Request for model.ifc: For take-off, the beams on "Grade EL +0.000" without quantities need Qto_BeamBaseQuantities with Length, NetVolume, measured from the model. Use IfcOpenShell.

First a look at what the model holds.

```python
import ifcopenshell
import ifcopenshell.util.element
import ifcopenshell.util.unit

model = ifcopenshell.open("model.ifc")
print(model.schema)
for unit_type in ("LENGTHUNIT", "AREAUNIT", "VOLUMEUNIT"):
    print(unit_type, ifcopenshell.util.unit.calculate_unit_scale(model, unit_type))
storey = next(s for s in model.by_type("IfcBuildingStorey") if s.Name == "Grade EL +0.000")
beams = [e for e in ifcopenshell.util.element.get_decomposition(storey) if e.is_a("IfcBeam")]
for e in sorted(beams, key=lambda e: e.id()):
    print(e.id(), e.is_a(), e.Name, list(ifcopenshell.util.element.get_psets(e, qtos_only=True)), sep=" | ")
```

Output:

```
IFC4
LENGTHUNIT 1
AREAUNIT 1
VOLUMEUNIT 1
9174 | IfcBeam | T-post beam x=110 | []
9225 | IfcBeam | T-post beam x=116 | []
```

```python
import ifcopenshell
import ifcopenshell.api.pset
import ifcopenshell.geom
import ifcopenshell.util.element
import ifcopenshell.util.shape
import ifcopenshell.util.unit

model = ifcopenshell.open("model.ifc")
unit_scale = ifcopenshell.util.unit.calculate_unit_scale(model)
volume_scale = ifcopenshell.util.unit.calculate_unit_scale(model, "VOLUMEUNIT")
settings = ifcopenshell.geom.settings()

storey = next(s for s in model.by_type("IfcBuildingStorey") if s.Name == "Grade EL +0.000")
beams = [e for e in ifcopenshell.util.element.get_decomposition(storey) if e.is_a("IfcBeam")]

for e in sorted(beams, key=lambda e: e.id()):
    if ifcopenshell.util.element.get_psets(e, qtos_only=True, should_inherit=False):
        continue
    # Geometry comes back in metres, in the element's own axes.
    shape = ifcopenshell.geom.create_shape(settings, e)
    values = {
        "Length": ifcopenshell.util.shape.get_max_xyz(shape.geometry) / unit_scale,
        "NetVolume": ifcopenshell.util.shape.get_volume(shape.geometry) / volume_scale,
    }
    qto = ifcopenshell.api.pset.add_qto(model, product=e, name="Qto_BeamBaseQuantities")
    ifcopenshell.api.pset.edit_qto(model, qto=qto, properties=values)
    print(e.id(), {k: round(v, 3) for k, v in values.items()})

model.write("model-out.ifc")
```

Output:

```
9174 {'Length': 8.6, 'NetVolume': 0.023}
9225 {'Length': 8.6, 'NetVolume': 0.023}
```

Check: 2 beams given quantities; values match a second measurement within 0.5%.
